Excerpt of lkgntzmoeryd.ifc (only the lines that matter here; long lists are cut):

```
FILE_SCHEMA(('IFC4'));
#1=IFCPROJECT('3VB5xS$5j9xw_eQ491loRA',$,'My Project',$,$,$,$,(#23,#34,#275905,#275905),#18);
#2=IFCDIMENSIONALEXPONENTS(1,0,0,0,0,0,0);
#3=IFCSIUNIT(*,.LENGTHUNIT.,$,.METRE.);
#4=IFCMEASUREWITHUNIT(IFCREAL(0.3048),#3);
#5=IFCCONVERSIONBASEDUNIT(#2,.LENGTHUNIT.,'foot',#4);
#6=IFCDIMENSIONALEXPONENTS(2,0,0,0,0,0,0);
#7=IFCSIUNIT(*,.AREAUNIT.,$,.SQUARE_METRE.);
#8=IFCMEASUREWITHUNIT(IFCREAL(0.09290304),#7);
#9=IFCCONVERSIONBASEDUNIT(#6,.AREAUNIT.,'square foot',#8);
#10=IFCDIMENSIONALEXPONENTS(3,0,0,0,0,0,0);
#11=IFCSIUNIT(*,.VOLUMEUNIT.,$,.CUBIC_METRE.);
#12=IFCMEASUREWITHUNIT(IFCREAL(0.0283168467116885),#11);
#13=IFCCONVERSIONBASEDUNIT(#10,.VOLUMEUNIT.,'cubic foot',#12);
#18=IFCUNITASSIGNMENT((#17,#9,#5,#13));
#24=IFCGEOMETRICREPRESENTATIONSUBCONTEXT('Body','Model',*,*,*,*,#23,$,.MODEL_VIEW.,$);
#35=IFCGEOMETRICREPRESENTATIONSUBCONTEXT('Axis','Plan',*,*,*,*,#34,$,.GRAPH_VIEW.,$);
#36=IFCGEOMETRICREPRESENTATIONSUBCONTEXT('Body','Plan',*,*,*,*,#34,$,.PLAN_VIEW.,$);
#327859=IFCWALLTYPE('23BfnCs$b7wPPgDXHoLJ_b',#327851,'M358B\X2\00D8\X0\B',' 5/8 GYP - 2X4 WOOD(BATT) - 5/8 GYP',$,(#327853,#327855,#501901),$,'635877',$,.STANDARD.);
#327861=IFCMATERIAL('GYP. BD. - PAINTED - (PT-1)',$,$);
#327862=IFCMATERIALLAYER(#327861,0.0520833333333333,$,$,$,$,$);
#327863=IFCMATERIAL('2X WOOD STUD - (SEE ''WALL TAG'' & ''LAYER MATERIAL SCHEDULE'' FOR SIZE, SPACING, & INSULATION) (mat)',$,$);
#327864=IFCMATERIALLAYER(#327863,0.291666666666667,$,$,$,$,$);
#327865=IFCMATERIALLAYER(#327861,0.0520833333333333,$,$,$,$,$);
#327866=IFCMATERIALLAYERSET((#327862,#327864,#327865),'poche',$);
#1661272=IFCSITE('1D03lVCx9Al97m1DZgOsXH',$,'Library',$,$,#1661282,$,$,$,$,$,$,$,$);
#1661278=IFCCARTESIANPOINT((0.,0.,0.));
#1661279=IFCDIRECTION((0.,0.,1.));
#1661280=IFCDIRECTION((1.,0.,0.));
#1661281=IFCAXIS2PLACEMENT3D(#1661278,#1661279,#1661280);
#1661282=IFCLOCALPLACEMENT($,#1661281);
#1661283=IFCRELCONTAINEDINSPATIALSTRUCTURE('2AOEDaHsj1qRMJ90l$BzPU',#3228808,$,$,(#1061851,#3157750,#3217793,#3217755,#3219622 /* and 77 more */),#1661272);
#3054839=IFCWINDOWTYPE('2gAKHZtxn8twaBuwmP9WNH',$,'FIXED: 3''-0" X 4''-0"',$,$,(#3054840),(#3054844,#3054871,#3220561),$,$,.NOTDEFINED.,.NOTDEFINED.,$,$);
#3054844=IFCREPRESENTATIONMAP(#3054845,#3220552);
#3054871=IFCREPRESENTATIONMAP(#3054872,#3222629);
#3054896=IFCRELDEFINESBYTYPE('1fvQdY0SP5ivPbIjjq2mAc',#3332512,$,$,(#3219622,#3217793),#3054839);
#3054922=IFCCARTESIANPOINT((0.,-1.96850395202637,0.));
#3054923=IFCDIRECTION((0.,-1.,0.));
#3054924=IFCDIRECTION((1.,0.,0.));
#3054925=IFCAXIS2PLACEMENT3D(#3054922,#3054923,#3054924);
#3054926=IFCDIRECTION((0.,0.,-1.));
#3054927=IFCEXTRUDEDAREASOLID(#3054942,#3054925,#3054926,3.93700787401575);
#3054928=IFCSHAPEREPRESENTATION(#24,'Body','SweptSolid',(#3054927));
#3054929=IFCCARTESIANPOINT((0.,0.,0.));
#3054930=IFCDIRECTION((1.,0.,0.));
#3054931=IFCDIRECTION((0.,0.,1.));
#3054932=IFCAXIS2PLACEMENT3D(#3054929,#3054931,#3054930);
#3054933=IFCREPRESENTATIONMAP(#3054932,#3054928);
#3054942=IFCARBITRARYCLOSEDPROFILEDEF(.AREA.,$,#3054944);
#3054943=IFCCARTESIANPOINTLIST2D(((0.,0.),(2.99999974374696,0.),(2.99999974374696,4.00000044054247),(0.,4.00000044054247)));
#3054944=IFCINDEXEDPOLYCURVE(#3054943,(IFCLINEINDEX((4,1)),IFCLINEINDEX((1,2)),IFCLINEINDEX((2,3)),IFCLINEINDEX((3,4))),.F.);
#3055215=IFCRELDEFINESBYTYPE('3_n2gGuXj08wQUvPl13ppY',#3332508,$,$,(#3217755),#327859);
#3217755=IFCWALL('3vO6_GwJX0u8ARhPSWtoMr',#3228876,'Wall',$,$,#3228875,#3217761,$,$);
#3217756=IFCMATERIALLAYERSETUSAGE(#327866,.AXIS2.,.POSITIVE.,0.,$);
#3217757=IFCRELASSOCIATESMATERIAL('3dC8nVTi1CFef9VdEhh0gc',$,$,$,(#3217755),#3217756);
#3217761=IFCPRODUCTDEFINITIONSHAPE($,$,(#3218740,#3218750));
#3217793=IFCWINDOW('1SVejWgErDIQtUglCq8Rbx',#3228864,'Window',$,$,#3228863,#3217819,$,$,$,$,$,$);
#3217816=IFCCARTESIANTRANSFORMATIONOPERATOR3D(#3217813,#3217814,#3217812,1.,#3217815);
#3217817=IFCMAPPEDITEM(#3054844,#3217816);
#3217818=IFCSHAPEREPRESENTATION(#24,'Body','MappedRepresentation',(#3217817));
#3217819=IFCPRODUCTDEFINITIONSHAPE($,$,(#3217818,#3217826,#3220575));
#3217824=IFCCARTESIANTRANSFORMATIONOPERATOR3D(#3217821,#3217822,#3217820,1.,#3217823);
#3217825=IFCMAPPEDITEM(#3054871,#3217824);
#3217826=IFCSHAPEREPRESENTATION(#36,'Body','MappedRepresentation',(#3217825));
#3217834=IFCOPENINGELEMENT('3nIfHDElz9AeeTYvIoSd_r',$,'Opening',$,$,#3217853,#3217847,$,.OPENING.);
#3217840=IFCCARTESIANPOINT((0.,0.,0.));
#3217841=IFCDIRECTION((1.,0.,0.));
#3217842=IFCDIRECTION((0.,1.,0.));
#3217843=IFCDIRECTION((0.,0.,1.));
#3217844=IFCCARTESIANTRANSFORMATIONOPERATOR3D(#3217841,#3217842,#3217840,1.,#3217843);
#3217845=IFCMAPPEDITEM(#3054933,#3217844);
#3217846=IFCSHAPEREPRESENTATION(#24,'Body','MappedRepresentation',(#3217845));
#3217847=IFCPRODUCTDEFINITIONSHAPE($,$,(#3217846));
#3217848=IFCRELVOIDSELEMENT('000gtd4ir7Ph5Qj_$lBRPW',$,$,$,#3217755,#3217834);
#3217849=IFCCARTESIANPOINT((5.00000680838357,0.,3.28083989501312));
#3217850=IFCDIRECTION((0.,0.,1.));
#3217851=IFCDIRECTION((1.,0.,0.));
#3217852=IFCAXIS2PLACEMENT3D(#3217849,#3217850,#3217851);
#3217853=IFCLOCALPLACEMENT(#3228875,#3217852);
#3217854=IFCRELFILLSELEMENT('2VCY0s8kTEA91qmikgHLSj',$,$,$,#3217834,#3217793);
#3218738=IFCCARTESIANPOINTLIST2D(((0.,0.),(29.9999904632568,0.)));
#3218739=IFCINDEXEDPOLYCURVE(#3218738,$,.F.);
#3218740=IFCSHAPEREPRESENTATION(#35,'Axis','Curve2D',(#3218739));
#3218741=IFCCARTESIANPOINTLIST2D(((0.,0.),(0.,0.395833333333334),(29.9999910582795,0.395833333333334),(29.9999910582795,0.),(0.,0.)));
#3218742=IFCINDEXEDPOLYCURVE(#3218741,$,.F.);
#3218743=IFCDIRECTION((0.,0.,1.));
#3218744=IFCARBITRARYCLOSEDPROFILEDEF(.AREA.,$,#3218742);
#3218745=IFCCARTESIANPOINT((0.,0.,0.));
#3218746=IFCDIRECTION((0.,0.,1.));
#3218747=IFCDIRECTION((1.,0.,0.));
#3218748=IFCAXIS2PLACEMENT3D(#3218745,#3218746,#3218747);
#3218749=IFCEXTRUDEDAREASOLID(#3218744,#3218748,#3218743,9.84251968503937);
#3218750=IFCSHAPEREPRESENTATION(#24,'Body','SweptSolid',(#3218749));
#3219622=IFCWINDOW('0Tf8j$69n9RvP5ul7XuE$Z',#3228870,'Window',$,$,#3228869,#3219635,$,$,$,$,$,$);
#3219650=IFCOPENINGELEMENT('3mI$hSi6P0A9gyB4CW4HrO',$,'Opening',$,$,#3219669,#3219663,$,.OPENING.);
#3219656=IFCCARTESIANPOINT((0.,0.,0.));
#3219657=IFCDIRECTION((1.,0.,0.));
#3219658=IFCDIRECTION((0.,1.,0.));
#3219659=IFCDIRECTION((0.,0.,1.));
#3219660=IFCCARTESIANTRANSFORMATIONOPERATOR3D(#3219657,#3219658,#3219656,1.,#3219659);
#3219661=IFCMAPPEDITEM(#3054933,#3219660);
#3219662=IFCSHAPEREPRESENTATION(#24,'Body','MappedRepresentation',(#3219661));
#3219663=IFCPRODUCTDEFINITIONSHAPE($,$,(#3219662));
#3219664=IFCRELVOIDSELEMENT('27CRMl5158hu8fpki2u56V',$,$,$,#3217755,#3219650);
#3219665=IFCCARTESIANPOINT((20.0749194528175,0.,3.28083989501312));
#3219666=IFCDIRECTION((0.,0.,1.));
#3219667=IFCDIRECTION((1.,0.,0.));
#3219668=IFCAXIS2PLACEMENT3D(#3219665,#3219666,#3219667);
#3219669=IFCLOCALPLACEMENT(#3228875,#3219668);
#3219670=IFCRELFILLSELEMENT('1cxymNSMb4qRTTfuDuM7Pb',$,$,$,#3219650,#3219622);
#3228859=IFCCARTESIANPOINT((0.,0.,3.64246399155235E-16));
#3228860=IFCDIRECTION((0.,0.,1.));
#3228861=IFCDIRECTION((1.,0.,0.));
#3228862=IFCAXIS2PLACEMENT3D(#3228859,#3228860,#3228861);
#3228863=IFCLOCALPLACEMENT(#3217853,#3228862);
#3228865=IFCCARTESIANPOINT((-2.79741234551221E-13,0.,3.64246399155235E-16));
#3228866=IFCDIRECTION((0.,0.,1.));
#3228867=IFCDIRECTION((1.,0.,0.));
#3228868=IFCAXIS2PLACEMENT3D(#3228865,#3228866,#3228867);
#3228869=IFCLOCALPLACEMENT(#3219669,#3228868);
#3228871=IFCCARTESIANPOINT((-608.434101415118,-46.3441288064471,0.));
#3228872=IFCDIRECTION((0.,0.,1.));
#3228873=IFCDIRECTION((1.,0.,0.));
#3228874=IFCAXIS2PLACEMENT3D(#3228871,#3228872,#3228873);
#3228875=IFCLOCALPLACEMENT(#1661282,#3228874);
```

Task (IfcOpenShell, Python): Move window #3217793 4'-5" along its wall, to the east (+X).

```python
import ifcopenshell
import ifcopenshell.api.geometry
import ifcopenshell.util.placement
import ifcopenshell.util.unit

model = ifcopenshell.open("lkgntzmoeryd.ifc")
unit_scale = ifcopenshell.util.unit.calculate_unit_scale(model)

window = model.by_guid("1SVejWgErDIQtUglCq8Rbx")
opening = window.FillsVoids[0].RelatingOpeningElement
wall = opening.VoidsElements[0].RelatingBuildingElement

wall_matrix = ifcopenshell.util.placement.get_local_placement(wall.ObjectPlacement)
shift = wall_matrix[:3, 0] * 53 * 0.0254 / unit_scale
before = ifcopenshell.util.placement.get_local_placement(window.ObjectPlacement)[:3, 3].copy()

# The window is placed relative to its opening, so it follows when the opening moves.
matrix = ifcopenshell.util.placement.get_local_placement(opening.ObjectPlacement)
matrix[:3, 3] += shift
ifcopenshell.api.geometry.edit_object_placement(
    model, product=opening, matrix=matrix, is_si=False, should_transform_children=True
)

after = ifcopenshell.util.placement.get_local_placement(window.ObjectPlacement)[:3, 3]
print("window moved by", (after - before).round(3) + 0.0)

model.write("lkgntzmoeryd_edited.ifc")
```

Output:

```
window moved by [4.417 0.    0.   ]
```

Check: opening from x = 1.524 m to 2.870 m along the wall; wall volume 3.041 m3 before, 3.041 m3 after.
